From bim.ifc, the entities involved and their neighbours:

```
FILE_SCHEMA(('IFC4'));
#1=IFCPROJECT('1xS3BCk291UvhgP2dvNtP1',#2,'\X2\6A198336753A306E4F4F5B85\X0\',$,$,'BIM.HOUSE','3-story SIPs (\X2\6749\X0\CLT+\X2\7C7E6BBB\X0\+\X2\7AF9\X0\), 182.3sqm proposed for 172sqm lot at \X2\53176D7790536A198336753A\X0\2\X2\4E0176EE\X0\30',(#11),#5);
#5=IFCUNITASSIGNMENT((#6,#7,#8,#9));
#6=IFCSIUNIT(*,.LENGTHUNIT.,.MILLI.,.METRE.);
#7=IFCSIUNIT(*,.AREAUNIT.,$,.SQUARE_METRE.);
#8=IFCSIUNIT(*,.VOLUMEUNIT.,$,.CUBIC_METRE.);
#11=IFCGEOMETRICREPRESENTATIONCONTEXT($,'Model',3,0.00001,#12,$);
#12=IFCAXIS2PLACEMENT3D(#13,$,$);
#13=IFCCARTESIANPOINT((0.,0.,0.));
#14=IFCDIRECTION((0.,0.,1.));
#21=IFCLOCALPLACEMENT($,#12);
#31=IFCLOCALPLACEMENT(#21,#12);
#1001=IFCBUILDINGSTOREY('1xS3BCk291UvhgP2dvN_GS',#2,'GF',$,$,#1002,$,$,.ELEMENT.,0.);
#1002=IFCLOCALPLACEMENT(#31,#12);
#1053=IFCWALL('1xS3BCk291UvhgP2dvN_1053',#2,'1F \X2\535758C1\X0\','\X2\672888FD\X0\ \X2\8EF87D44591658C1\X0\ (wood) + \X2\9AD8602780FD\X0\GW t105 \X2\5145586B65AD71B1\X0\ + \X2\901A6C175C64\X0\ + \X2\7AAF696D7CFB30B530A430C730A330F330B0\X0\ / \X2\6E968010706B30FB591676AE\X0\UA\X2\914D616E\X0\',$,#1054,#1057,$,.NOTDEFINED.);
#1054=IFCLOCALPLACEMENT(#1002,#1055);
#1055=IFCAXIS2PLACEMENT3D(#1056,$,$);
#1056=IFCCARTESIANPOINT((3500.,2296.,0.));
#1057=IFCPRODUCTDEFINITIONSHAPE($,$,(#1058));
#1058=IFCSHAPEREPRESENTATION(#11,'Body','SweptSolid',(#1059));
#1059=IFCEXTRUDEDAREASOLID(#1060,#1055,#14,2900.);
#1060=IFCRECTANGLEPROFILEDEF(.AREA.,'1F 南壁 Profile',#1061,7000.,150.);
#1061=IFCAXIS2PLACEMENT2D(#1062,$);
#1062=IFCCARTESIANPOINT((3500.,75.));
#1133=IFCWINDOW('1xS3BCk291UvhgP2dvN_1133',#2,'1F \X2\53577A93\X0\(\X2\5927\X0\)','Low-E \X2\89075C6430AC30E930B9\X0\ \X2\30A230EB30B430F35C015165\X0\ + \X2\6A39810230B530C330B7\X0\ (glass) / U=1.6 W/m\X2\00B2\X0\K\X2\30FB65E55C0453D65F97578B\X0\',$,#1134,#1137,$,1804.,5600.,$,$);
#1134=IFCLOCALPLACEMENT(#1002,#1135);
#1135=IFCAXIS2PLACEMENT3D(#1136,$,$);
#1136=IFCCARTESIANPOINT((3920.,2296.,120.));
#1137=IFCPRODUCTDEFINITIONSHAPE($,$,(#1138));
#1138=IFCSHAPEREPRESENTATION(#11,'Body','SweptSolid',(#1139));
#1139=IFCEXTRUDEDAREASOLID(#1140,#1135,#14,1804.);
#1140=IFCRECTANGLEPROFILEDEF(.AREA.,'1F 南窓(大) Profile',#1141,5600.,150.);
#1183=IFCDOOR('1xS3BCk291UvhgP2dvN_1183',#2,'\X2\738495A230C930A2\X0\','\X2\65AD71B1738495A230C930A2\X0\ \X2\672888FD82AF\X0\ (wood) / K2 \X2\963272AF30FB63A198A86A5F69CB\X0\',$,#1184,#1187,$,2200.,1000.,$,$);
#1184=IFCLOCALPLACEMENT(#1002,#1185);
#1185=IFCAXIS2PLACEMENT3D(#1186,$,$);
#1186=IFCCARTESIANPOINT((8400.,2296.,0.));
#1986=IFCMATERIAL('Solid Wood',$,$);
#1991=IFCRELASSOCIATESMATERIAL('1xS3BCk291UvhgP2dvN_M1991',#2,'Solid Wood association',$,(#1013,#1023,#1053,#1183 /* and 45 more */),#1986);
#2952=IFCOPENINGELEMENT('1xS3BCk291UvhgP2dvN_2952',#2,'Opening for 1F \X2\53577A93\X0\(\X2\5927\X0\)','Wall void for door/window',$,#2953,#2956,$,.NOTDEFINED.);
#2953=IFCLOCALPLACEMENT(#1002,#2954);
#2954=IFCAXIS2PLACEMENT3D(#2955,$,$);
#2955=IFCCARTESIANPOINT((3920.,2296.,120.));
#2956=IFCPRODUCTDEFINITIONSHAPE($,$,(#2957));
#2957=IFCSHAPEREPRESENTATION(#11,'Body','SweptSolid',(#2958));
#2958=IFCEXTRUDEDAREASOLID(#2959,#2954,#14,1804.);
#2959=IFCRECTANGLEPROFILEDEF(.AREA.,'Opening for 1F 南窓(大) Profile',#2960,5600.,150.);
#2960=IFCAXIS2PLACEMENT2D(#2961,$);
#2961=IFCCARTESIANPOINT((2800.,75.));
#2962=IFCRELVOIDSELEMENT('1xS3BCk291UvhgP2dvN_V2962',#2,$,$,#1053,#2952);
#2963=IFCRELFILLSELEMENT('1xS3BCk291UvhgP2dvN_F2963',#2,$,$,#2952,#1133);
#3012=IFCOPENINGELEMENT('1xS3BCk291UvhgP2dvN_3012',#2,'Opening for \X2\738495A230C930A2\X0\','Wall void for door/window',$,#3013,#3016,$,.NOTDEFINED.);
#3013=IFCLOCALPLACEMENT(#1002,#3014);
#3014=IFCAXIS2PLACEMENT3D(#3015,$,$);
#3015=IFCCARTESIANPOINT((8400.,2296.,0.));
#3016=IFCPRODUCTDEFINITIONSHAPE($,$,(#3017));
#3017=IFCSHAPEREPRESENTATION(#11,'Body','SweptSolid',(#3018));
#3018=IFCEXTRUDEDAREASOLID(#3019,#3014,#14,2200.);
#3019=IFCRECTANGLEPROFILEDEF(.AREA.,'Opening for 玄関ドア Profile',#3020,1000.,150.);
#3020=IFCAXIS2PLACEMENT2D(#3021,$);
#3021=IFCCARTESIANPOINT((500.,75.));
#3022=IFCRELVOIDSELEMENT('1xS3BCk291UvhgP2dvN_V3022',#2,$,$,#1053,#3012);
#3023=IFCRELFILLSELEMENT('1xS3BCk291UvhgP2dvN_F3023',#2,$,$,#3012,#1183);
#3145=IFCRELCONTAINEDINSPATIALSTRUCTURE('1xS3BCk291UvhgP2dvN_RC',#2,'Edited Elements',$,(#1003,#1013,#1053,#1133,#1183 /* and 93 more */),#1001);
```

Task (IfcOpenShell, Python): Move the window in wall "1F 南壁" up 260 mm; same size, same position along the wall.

```python
import numpy as np
import ifcopenshell
import ifcopenshell.api.geometry
import ifcopenshell.util.placement
import ifcopenshell.util.unit

model = ifcopenshell.open("bim.ifc")
unit_scale = ifcopenshell.util.unit.calculate_unit_scale(model)

window = model.by_id(1133)
opening = window.FillsVoids[0].RelatingOpeningElement
dz = 260.0

shift = np.array([0.0, 0.0, dz])
# The window is not placed relative to its opening, so move both.
for product in (opening, window):
    matrix = ifcopenshell.util.placement.get_local_placement(product.ObjectPlacement)
    matrix[:3, 3] += shift
    ifcopenshell.api.geometry.edit_object_placement(model, product=product, matrix=matrix, is_si=False)

print(f"moved by {dz * unit_scale:+.3f} m")

model.write("bim_v2.ifc")
```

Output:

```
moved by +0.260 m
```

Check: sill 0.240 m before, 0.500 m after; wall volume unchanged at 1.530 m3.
